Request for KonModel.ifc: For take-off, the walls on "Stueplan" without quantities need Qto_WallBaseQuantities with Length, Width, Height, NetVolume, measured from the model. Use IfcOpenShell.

First a look at what the model holds.

```python
import ifcopenshell
import ifcopenshell.util.element
import ifcopenshell.util.unit

model = ifcopenshell.open("KonModel.ifc")
print(model.schema)
for unit_type in ("LENGTHUNIT", "AREAUNIT", "VOLUMEUNIT"):
    print(unit_type, ifcopenshell.util.unit.calculate_unit_scale(model, unit_type))
storey = next(s for s in model.by_type("IfcBuildingStorey") if s.Name == "Stueplan")
walls = [e for e in ifcopenshell.util.element.get_decomposition(storey) if e.is_a("IfcWall")]
for e in sorted(walls, key=lambda e: e.id()):
    print(e.id(), e.is_a(), e.Name, list(ifcopenshell.util.element.get_psets(e, qtos_only=True)), sep=" | ")
```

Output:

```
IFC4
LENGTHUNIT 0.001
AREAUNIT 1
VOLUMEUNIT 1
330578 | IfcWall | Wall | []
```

```python
import ifcopenshell
import ifcopenshell.api.pset
import ifcopenshell.geom
import ifcopenshell.util.element
import ifcopenshell.util.shape
import ifcopenshell.util.unit

model = ifcopenshell.open("KonModel.ifc")
unit_scale = ifcopenshell.util.unit.calculate_unit_scale(model)
volume_scale = ifcopenshell.util.unit.calculate_unit_scale(model, "VOLUMEUNIT")
settings = ifcopenshell.geom.settings()

storey = next(s for s in model.by_type("IfcBuildingStorey") if s.Name == "Stueplan")
walls = [e for e in ifcopenshell.util.element.get_decomposition(storey) if e.is_a("IfcWall")]

for e in sorted(walls, key=lambda e: e.id()):
    if ifcopenshell.util.element.get_psets(e, qtos_only=True, should_inherit=False):
        continue
    # Geometry comes back in metres, in the element's own axes.
    shape = ifcopenshell.geom.create_shape(settings, e)
    values = {
        "Length": ifcopenshell.util.shape.get_x(shape.geometry) / unit_scale,
        "Width": ifcopenshell.util.shape.get_y(shape.geometry) / unit_scale,
        "Height": ifcopenshell.util.shape.get_z(shape.geometry) / unit_scale,
        "NetVolume": ifcopenshell.util.shape.get_volume(shape.geometry) / volume_scale,
    }
    qto = ifcopenshell.api.pset.add_qto(model, product=e, name="Qto_WallBaseQuantities")
    ifcopenshell.api.pset.edit_qto(model, qto=qto, properties=values)
    print(e.id(), {k: round(v, 3) for k, v in values.items()})

model.write("KonModel_rev.ifc")
```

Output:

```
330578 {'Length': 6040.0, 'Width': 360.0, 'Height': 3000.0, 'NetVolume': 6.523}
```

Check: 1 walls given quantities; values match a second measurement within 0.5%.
